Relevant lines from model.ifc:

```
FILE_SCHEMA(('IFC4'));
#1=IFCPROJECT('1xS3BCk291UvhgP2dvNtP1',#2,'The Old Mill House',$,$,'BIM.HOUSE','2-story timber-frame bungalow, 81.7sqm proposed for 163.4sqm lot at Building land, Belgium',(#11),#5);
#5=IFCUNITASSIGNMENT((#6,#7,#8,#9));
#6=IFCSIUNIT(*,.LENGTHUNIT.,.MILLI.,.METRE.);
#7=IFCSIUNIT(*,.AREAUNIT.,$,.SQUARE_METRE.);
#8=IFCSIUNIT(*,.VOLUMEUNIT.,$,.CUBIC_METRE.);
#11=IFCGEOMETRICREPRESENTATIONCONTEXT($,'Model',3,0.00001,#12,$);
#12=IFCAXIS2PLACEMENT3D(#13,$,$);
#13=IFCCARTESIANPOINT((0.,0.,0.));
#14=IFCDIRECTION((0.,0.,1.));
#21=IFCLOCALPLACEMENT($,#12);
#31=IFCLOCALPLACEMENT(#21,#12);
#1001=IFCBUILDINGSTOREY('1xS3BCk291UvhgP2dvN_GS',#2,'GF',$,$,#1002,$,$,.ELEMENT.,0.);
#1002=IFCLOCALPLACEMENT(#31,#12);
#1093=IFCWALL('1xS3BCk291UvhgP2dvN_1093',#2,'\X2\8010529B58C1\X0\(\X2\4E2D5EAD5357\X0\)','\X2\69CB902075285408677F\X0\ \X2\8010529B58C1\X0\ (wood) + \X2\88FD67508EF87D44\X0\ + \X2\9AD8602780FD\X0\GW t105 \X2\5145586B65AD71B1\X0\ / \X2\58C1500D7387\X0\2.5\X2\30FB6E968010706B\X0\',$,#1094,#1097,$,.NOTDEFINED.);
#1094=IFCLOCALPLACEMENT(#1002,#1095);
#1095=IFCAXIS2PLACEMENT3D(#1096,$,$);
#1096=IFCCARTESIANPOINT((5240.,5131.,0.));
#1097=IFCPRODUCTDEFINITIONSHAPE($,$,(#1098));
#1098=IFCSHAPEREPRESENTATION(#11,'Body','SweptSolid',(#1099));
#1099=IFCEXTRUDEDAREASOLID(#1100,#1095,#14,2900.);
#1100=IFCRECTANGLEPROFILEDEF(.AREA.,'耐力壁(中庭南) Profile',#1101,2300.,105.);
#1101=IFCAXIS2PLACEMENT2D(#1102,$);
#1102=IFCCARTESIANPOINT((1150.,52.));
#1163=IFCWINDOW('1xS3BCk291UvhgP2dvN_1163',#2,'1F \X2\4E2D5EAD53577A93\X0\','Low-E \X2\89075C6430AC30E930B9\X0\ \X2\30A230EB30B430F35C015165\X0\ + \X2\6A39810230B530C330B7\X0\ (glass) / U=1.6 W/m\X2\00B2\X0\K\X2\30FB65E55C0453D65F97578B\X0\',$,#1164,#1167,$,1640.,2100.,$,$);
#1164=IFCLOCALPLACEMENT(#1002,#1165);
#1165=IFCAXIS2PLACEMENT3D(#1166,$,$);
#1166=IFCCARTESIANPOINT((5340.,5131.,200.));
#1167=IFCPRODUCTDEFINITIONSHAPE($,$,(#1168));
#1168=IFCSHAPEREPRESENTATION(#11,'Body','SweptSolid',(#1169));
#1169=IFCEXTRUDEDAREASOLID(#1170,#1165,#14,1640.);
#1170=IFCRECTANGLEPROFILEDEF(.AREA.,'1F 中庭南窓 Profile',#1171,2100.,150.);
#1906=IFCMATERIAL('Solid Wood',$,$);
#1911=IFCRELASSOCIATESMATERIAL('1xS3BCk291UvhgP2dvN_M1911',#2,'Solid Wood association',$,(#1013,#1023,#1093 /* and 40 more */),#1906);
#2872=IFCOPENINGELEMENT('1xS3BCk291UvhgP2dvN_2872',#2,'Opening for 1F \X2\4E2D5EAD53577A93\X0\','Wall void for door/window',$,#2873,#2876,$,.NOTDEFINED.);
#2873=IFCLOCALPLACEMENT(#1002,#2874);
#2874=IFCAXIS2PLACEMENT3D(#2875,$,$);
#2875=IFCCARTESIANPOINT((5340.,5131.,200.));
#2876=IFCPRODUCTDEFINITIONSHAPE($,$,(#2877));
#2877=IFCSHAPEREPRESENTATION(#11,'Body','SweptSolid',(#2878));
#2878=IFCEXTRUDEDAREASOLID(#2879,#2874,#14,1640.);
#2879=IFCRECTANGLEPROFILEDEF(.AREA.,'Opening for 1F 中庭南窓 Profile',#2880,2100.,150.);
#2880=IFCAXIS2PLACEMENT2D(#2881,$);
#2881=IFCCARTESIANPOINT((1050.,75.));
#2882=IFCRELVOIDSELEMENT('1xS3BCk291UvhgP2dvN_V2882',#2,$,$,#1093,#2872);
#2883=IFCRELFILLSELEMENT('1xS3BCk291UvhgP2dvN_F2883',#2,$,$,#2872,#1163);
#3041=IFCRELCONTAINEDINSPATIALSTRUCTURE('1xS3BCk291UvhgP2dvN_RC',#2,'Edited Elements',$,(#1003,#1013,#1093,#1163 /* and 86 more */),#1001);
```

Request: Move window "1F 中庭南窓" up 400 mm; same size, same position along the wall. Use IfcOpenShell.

```python
import numpy as np
import ifcopenshell
import ifcopenshell.api.geometry
import ifcopenshell.util.placement
import ifcopenshell.util.unit

model = ifcopenshell.open("model.ifc")
unit_scale = ifcopenshell.util.unit.calculate_unit_scale(model)

window = model.by_guid("1xS3BCk291UvhgP2dvN_1163")
opening = window.FillsVoids[0].RelatingOpeningElement
dz = 400.0

shift = np.array([0.0, 0.0, dz])
# The window is not placed relative to its opening, so move both.
for product in (opening, window):
    matrix = ifcopenshell.util.placement.get_local_placement(product.ObjectPlacement)
    matrix[:3, 3] += shift
    ifcopenshell.api.geometry.edit_object_placement(model, product=product, matrix=matrix, is_si=False)

print(f"moved by {dz * unit_scale:+.3f} m")

model.write("model_updated.ifc")
```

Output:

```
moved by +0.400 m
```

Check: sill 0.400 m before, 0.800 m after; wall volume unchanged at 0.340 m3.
